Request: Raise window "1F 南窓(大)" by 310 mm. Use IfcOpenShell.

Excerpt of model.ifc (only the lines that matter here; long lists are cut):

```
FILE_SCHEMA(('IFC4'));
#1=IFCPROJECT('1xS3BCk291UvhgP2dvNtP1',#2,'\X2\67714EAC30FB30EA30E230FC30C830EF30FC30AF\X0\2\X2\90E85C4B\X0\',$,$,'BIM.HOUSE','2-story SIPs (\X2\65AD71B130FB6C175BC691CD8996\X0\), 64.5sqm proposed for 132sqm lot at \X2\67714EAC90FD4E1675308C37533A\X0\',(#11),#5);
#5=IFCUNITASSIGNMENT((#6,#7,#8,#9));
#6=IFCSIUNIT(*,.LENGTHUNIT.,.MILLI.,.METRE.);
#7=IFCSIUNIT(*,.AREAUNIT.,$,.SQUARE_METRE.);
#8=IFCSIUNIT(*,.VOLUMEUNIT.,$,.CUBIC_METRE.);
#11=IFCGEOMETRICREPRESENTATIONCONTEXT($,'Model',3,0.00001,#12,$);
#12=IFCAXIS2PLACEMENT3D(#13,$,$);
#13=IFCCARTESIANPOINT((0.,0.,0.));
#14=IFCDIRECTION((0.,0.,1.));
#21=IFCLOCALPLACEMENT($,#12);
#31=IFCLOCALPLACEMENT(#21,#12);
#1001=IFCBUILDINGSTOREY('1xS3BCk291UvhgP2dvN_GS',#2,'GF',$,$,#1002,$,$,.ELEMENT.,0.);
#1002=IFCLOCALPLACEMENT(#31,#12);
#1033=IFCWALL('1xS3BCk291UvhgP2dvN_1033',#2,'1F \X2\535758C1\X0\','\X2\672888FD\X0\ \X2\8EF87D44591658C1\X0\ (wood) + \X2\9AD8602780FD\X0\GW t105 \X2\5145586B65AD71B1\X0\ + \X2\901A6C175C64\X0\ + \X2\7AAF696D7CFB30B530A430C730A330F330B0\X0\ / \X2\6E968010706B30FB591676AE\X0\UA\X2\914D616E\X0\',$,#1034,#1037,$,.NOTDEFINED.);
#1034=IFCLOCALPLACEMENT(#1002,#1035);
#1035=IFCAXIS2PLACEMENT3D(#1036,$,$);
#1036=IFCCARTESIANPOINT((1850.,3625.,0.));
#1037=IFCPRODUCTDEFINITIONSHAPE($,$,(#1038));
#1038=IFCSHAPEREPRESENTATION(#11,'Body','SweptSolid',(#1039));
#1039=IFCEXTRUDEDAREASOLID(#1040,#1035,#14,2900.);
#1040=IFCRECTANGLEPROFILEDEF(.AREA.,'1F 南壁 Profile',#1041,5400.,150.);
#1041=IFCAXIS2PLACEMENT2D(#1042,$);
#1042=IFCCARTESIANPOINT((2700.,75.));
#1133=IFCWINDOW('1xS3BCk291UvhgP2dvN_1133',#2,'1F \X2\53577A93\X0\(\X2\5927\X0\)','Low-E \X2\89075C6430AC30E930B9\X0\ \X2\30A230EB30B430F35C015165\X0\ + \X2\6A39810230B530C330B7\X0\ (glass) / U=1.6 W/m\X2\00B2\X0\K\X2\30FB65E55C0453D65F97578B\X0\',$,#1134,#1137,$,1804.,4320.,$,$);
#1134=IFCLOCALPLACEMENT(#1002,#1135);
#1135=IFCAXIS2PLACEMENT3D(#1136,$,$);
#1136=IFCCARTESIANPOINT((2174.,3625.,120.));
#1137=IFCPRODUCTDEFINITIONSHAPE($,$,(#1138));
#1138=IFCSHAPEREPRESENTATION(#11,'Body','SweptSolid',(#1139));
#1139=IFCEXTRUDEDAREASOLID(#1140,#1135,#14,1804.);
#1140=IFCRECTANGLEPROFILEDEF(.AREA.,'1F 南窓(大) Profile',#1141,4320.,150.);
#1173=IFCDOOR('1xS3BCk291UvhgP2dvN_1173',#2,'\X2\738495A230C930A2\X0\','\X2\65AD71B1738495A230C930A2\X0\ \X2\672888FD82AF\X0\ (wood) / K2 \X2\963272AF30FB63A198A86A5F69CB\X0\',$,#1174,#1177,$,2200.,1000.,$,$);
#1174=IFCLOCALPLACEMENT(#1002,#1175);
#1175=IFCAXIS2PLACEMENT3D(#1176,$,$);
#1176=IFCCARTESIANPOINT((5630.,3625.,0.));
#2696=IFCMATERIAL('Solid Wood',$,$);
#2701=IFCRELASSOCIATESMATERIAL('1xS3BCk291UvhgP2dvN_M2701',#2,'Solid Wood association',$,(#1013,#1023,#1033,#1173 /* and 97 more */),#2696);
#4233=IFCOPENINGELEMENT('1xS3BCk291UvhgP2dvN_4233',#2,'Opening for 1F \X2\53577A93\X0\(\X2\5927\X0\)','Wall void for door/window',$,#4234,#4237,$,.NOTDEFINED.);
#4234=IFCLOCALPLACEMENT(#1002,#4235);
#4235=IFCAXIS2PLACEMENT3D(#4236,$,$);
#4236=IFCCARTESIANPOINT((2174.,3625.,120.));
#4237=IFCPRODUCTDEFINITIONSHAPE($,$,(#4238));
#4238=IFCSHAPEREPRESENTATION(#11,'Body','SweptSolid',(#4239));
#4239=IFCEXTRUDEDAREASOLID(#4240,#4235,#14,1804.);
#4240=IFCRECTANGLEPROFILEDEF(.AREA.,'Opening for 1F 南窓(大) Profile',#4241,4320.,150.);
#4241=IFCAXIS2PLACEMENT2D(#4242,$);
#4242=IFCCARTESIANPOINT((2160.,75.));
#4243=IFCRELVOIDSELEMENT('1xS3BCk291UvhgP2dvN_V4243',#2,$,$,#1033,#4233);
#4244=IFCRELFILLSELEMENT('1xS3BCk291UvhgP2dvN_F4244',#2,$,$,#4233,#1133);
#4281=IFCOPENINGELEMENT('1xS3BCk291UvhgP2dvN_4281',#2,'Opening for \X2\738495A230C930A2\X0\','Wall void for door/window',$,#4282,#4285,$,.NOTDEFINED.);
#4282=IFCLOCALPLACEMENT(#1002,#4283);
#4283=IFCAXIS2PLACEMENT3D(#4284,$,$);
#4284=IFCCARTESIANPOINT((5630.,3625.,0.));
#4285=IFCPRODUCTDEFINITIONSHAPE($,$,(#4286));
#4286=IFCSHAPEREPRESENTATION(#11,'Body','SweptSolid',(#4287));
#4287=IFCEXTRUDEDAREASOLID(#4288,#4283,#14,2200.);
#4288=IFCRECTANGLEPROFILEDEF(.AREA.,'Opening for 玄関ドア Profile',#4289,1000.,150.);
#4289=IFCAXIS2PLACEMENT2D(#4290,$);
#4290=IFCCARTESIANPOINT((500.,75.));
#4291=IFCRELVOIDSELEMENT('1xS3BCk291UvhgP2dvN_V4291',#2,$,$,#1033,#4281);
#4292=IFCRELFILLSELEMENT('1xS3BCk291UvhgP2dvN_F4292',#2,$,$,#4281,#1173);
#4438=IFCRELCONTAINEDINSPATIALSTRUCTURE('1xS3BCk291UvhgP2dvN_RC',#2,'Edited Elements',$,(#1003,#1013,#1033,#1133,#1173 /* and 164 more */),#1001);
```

```python
import numpy as np
import ifcopenshell
import ifcopenshell.api.geometry
import ifcopenshell.util.placement
import ifcopenshell.util.unit

model = ifcopenshell.open("model.ifc")
unit_scale = ifcopenshell.util.unit.calculate_unit_scale(model)

window = model.by_guid("1xS3BCk291UvhgP2dvN_1133")
opening = window.FillsVoids[0].RelatingOpeningElement
dz = 0.31 / unit_scale

shift = np.array([0.0, 0.0, dz])
# The window is not placed relative to its opening, so move both.
for product in (opening, window):
    matrix = ifcopenshell.util.placement.get_local_placement(product.ObjectPlacement)
    matrix[:3, 3] += shift
    ifcopenshell.api.geometry.edit_object_placement(model, product=product, matrix=matrix, is_si=False)

print(f"moved by {dz * unit_scale:+.3f} m")

model.write("model-out.ifc")
```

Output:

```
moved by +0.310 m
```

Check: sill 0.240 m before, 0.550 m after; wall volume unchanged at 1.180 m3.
